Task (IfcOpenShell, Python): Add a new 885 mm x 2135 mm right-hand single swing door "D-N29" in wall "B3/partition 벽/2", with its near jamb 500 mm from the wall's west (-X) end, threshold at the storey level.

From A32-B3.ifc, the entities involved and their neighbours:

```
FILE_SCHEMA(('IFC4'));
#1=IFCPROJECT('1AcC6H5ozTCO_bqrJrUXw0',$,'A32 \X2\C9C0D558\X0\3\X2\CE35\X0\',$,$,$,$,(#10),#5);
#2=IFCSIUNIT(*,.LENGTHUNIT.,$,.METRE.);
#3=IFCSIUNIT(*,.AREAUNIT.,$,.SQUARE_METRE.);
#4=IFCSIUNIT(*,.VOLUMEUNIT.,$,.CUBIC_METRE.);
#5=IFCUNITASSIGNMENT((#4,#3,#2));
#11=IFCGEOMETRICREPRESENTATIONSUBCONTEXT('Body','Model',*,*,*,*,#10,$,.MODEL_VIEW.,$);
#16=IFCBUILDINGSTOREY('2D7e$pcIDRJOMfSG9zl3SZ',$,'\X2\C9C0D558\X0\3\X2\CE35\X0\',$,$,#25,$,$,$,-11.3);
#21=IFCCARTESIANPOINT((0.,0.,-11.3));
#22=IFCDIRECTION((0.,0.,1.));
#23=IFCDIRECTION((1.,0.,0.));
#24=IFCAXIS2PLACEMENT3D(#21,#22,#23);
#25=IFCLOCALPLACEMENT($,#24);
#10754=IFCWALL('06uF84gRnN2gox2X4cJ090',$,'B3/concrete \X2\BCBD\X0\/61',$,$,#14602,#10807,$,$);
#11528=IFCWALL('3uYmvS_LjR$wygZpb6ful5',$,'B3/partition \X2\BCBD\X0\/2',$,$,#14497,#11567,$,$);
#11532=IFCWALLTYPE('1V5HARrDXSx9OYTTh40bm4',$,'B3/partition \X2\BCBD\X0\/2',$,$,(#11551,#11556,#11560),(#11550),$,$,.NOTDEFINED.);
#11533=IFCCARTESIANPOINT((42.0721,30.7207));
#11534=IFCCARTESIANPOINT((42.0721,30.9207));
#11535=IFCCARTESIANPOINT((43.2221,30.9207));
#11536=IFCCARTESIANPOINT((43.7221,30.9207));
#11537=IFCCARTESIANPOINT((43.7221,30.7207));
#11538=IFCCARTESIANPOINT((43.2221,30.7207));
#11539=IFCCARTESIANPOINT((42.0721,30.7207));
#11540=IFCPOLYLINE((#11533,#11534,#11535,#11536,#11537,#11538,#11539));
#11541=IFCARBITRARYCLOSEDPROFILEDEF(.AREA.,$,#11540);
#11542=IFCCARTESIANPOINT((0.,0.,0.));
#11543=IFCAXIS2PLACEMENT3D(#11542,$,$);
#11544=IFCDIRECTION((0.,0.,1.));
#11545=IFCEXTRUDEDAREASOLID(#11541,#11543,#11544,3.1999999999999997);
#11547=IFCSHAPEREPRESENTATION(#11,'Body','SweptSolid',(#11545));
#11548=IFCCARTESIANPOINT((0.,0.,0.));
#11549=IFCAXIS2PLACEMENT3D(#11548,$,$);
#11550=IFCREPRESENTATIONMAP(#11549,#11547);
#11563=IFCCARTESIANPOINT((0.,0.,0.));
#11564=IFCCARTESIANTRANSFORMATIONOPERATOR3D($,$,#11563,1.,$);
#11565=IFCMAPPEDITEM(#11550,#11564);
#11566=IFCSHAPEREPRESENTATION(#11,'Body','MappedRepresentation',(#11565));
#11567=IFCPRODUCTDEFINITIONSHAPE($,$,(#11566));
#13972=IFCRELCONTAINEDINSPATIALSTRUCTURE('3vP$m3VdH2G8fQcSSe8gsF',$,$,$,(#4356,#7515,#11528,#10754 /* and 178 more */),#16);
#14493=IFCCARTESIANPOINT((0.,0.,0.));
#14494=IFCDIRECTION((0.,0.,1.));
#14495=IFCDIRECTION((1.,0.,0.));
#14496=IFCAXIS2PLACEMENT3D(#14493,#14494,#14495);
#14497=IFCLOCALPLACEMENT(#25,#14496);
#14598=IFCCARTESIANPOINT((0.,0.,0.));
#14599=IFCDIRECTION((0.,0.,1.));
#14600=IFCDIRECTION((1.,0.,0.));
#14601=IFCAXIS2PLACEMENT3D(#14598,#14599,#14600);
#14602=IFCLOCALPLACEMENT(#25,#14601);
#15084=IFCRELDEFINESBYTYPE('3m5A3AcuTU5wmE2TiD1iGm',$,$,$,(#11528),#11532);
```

```python
import numpy as np
import ifcopenshell
import ifcopenshell.api.feature
import ifcopenshell.api.geometry
import ifcopenshell.api.root
import ifcopenshell.api.spatial
import ifcopenshell.geom
import ifcopenshell.util.element
import ifcopenshell.util.placement
import ifcopenshell.util.representation
import ifcopenshell.util.shape
import ifcopenshell.util.unit

model = ifcopenshell.open("A32-B3.ifc")
unit_scale = ifcopenshell.util.unit.calculate_unit_scale(model)
settings = ifcopenshell.geom.settings()


def volume(element):
    """Net volume in cubic metres, openings subtracted."""
    shape = ifcopenshell.geom.create_shape(settings, element)
    return ifcopenshell.util.shape.get_volume(shape.geometry)


wall = model.by_guid("3uYmvS_LjR$wygZpb6ful5")
storey = ifcopenshell.util.element.get_container(wall, ifc_class="IfcBuildingStorey")
context = ifcopenshell.util.representation.get_context(model, "Model", "Body", "MODEL_VIEW")
before = volume(wall)

width, height, from_end, sill = 0.885, 2.135, 0.5, 0.0  # metres

# The wall runs along its own X axis, and the end named is its -X end.
wall_shape = ifcopenshell.geom.create_shape(settings, wall)
x, y, z = ifcopenshell.util.shape.get_vertices(wall_shape.geometry).T
start = x.min() + from_end
face, thickness = float(y.min()), float(y.max() - y.min())
wall_matrix = ifcopenshell.util.placement.get_local_placement(wall.ObjectPlacement)
level = ifcopenshell.util.placement.get_local_placement(storey.ObjectPlacement)[2, 3]


def in_wall(x, y):
    """Placement at x, y metres in the wall's axes, at sill height."""
    matrix = wall_matrix.copy()
    matrix[:, 3] = wall_matrix @ np.array([x / unit_scale, y / unit_scale, 0.0, 1.0])
    matrix[2, 3] = level + sill / unit_scale
    return matrix


# Opening: a box that overshoots both wall faces by 50 mm.
opening = ifcopenshell.api.root.create_entity(model, ifc_class="IfcOpeningElement", predefined_type="OPENING")
box = ifcopenshell.api.geometry.add_wall_representation(
    model, context=context, length=width, height=height, thickness=thickness + 0.1
)
ifcopenshell.api.geometry.assign_representation(model, product=opening, representation=box)
ifcopenshell.api.geometry.edit_object_placement(model, product=opening, matrix=in_wall(start, face - 0.05), is_si=False)
ifcopenshell.api.feature.add_feature(model, feature=opening, element=wall)

door = ifcopenshell.api.root.create_entity(model, ifc_class="IfcDoor", name="D-N29", predefined_type="DOOR")
door.OverallWidth, door.OverallHeight = width / unit_scale, height / unit_scale
door.OperationType = "SINGLE_SWING_RIGHT"
body = ifcopenshell.api.geometry.add_door_representation(
    model,
    context=context,
    overall_width=door.OverallWidth,
    overall_height=door.OverallHeight,
    operation_type="SINGLE_SWING_RIGHT",
    lining_properties={"LiningDepth": thickness / unit_scale, "ThresholdDepth": thickness / unit_scale},
)
ifcopenshell.api.geometry.assign_representation(model, product=door, representation=body)
ifcopenshell.api.spatial.assign_container(model, products=[door], relating_structure=storey)
ifcopenshell.api.feature.add_filling(model, opening=opening, element=door)

# The lining spans the wall, so the door starts at the wall face.
ifcopenshell.api.geometry.edit_object_placement(model, product=door, matrix=in_wall(start, face), is_si=False)

after = volume(wall)

print(f"wall volume {before:.3f} -> {after:.3f} m3")

model.write("A32-B3_rev.ifc")
```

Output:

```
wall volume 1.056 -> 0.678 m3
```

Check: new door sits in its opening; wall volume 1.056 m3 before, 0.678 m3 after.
